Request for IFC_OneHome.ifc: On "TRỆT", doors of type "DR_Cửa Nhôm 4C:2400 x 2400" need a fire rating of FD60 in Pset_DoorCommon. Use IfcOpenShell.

First a look at what the model holds.

```python
import ifcopenshell
import ifcopenshell.util.element

model = ifcopenshell.open("IFC_OneHome.ifc")
print(model.schema)
storey = next(s for s in model.by_type("IfcBuildingStorey") if s.Name == "TRỆT")
doors = [e for e in ifcopenshell.util.element.get_decomposition(storey) if e.is_a("IfcDoor")]
seen = {}
for e in doors:
    element_type = ifcopenshell.util.element.get_type(e)
    key = (element_type.Name if element_type != e and element_type else None, ifcopenshell.util.element.get_pset(e, "Pset_DoorCommon", "FireRating"))
    seen[key] = seen.get(key, 0) + 1
for (name, value), count in sorted(seen.items(), key=str):
    print(count, "x", name, "|", value)
```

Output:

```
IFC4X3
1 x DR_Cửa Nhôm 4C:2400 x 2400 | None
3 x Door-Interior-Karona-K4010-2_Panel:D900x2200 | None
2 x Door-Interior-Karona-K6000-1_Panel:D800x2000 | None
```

```python
import ifcopenshell
import ifcopenshell.api.pset
import ifcopenshell.util.element

model = ifcopenshell.open("IFC_OneHome.ifc")

storey = next(s for s in model.by_type("IfcBuildingStorey") if s.Name == "TRỆT")
doors = [e for e in ifcopenshell.util.element.get_decomposition(storey) if e.is_a("IfcDoor")]

count = 0
for e in doors:
    element_type = ifcopenshell.util.element.get_type(e)
    if element_type in (None, e) or element_type.Name != "DR_Cửa Nhôm 4C:2400 x 2400":
        continue
    # add_pset returns the element's existing set when there is one.
    pset = ifcopenshell.api.pset.add_pset(model, product=e, name="Pset_DoorCommon")
    ifcopenshell.api.pset.edit_pset(model, pset=pset, properties={"FireRating": "FD60"})
    count += 1

print(count, "doors updated")

model.write("IFC_OneHome-out.ifc")
```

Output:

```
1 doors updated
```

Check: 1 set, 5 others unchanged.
